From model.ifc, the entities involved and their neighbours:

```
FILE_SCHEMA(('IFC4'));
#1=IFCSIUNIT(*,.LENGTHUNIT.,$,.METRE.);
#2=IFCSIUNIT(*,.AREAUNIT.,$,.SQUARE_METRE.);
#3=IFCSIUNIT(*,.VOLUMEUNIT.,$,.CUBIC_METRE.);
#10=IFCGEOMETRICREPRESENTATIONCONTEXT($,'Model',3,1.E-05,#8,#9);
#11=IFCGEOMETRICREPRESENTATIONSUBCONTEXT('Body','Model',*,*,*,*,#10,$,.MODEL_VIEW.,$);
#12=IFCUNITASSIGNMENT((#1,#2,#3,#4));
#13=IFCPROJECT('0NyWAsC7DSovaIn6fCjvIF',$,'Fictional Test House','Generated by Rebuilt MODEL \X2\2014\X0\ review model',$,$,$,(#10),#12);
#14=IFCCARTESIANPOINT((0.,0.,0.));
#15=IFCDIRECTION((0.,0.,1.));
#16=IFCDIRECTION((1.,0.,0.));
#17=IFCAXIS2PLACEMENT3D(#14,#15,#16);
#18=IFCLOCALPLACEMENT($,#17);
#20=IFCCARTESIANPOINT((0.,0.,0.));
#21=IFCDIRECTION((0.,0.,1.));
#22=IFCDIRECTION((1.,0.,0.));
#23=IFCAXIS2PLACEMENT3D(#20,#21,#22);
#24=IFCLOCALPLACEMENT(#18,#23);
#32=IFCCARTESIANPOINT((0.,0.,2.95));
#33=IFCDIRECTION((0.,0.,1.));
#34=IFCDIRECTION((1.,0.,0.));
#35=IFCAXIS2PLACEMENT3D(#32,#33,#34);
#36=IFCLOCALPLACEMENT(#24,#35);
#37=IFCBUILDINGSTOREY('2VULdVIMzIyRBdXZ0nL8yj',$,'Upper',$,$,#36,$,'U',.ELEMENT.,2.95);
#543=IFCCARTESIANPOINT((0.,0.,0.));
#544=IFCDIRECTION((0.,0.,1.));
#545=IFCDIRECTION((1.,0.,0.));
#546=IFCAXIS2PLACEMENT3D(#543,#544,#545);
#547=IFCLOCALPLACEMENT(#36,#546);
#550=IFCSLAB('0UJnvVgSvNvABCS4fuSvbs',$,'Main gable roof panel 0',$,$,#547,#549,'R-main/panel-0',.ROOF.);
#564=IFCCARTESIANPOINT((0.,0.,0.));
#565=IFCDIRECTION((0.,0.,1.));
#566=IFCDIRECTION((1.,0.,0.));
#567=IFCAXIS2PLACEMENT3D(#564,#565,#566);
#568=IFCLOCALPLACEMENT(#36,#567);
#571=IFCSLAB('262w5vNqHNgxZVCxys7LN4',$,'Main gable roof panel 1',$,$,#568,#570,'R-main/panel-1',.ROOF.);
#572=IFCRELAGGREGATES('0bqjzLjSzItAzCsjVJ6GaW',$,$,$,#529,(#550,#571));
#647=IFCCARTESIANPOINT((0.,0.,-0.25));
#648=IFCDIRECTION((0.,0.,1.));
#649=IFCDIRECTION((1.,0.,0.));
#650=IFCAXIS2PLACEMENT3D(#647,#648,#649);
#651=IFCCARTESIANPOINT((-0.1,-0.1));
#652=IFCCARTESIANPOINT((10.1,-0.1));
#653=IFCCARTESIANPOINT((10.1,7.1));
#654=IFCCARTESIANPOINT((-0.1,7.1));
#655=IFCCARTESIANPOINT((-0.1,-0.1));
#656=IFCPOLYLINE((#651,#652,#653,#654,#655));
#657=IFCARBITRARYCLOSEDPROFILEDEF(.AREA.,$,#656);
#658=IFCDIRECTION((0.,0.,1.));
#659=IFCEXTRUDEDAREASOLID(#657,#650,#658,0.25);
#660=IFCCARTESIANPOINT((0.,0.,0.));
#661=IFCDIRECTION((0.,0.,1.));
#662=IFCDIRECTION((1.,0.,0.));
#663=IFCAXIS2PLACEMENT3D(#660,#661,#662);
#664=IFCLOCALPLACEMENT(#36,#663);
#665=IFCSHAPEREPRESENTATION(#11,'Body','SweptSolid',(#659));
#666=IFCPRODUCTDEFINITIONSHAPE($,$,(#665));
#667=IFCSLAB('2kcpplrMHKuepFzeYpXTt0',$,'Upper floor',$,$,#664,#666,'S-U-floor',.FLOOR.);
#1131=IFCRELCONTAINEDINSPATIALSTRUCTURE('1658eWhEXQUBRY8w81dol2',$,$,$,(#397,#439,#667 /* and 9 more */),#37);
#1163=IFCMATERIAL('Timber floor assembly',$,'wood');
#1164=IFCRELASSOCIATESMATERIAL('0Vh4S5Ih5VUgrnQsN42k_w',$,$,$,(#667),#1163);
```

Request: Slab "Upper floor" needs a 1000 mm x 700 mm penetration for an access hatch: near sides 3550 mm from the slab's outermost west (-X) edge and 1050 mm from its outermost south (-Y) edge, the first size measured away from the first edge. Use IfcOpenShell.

```python
import numpy as np
import ifcopenshell
import ifcopenshell.api.feature
import ifcopenshell.api.geometry
import ifcopenshell.api.root
import ifcopenshell.geom
import ifcopenshell.util.placement
import ifcopenshell.util.representation
import ifcopenshell.util.shape
import ifcopenshell.util.unit

model = ifcopenshell.open("model.ifc")
unit_scale = ifcopenshell.util.unit.calculate_unit_scale(model)
settings = ifcopenshell.geom.settings()


def volume(element):
    """Net volume in cubic metres, openings subtracted."""
    shape = ifcopenshell.geom.create_shape(settings, element)
    return ifcopenshell.util.shape.get_volume(shape.geometry)


slab = model.by_guid("2kcpplrMHKuepFzeYpXTt0")
before = volume(slab)

# Extent in the slab's own axes, in metres. The edges named are its -X and -Y sides.
slab_shape = ifcopenshell.geom.create_shape(settings, slab)
vertices = ifcopenshell.util.shape.get_vertices(slab_shape.geometry)
x_min, y_min, bottom = vertices.min(axis=0)
top = vertices[:, 2].max()

opening = ifcopenshell.api.root.create_entity(model, ifc_class="IfcOpeningElement", name="Access hatch opening", predefined_type="OPENING")
context = ifcopenshell.util.representation.get_context(model, "Model", "Body", "MODEL_VIEW")
width, depth = 1, 0.7
outline = [(0.0, 0.0), (width, 0.0), (width, depth), (0.0, depth), (0.0, 0.0)]
# Overshoot both faces by 50 mm so the cut is clean.
shape = ifcopenshell.api.geometry.add_slab_representation(
    model, context=context, depth=top - bottom + 0.1, polyline=outline
)
ifcopenshell.api.geometry.assign_representation(model, product=opening, representation=shape)

matrix = ifcopenshell.util.placement.get_local_placement(slab.ObjectPlacement)
matrix[:, 3] = matrix @ np.append(np.array([x_min + 3.55, y_min + 1.05, bottom - 0.05]) / unit_scale, 1.0)
ifcopenshell.api.geometry.edit_object_placement(model, product=opening, matrix=matrix, is_si=False)
ifcopenshell.api.feature.add_feature(model, feature=opening, element=slab)

after = volume(slab)

print(f"slab volume {before:.3f} -> {after:.3f} m3")

model.write("model_edited.ifc")
```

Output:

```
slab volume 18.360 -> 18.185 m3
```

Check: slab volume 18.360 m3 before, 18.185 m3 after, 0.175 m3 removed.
